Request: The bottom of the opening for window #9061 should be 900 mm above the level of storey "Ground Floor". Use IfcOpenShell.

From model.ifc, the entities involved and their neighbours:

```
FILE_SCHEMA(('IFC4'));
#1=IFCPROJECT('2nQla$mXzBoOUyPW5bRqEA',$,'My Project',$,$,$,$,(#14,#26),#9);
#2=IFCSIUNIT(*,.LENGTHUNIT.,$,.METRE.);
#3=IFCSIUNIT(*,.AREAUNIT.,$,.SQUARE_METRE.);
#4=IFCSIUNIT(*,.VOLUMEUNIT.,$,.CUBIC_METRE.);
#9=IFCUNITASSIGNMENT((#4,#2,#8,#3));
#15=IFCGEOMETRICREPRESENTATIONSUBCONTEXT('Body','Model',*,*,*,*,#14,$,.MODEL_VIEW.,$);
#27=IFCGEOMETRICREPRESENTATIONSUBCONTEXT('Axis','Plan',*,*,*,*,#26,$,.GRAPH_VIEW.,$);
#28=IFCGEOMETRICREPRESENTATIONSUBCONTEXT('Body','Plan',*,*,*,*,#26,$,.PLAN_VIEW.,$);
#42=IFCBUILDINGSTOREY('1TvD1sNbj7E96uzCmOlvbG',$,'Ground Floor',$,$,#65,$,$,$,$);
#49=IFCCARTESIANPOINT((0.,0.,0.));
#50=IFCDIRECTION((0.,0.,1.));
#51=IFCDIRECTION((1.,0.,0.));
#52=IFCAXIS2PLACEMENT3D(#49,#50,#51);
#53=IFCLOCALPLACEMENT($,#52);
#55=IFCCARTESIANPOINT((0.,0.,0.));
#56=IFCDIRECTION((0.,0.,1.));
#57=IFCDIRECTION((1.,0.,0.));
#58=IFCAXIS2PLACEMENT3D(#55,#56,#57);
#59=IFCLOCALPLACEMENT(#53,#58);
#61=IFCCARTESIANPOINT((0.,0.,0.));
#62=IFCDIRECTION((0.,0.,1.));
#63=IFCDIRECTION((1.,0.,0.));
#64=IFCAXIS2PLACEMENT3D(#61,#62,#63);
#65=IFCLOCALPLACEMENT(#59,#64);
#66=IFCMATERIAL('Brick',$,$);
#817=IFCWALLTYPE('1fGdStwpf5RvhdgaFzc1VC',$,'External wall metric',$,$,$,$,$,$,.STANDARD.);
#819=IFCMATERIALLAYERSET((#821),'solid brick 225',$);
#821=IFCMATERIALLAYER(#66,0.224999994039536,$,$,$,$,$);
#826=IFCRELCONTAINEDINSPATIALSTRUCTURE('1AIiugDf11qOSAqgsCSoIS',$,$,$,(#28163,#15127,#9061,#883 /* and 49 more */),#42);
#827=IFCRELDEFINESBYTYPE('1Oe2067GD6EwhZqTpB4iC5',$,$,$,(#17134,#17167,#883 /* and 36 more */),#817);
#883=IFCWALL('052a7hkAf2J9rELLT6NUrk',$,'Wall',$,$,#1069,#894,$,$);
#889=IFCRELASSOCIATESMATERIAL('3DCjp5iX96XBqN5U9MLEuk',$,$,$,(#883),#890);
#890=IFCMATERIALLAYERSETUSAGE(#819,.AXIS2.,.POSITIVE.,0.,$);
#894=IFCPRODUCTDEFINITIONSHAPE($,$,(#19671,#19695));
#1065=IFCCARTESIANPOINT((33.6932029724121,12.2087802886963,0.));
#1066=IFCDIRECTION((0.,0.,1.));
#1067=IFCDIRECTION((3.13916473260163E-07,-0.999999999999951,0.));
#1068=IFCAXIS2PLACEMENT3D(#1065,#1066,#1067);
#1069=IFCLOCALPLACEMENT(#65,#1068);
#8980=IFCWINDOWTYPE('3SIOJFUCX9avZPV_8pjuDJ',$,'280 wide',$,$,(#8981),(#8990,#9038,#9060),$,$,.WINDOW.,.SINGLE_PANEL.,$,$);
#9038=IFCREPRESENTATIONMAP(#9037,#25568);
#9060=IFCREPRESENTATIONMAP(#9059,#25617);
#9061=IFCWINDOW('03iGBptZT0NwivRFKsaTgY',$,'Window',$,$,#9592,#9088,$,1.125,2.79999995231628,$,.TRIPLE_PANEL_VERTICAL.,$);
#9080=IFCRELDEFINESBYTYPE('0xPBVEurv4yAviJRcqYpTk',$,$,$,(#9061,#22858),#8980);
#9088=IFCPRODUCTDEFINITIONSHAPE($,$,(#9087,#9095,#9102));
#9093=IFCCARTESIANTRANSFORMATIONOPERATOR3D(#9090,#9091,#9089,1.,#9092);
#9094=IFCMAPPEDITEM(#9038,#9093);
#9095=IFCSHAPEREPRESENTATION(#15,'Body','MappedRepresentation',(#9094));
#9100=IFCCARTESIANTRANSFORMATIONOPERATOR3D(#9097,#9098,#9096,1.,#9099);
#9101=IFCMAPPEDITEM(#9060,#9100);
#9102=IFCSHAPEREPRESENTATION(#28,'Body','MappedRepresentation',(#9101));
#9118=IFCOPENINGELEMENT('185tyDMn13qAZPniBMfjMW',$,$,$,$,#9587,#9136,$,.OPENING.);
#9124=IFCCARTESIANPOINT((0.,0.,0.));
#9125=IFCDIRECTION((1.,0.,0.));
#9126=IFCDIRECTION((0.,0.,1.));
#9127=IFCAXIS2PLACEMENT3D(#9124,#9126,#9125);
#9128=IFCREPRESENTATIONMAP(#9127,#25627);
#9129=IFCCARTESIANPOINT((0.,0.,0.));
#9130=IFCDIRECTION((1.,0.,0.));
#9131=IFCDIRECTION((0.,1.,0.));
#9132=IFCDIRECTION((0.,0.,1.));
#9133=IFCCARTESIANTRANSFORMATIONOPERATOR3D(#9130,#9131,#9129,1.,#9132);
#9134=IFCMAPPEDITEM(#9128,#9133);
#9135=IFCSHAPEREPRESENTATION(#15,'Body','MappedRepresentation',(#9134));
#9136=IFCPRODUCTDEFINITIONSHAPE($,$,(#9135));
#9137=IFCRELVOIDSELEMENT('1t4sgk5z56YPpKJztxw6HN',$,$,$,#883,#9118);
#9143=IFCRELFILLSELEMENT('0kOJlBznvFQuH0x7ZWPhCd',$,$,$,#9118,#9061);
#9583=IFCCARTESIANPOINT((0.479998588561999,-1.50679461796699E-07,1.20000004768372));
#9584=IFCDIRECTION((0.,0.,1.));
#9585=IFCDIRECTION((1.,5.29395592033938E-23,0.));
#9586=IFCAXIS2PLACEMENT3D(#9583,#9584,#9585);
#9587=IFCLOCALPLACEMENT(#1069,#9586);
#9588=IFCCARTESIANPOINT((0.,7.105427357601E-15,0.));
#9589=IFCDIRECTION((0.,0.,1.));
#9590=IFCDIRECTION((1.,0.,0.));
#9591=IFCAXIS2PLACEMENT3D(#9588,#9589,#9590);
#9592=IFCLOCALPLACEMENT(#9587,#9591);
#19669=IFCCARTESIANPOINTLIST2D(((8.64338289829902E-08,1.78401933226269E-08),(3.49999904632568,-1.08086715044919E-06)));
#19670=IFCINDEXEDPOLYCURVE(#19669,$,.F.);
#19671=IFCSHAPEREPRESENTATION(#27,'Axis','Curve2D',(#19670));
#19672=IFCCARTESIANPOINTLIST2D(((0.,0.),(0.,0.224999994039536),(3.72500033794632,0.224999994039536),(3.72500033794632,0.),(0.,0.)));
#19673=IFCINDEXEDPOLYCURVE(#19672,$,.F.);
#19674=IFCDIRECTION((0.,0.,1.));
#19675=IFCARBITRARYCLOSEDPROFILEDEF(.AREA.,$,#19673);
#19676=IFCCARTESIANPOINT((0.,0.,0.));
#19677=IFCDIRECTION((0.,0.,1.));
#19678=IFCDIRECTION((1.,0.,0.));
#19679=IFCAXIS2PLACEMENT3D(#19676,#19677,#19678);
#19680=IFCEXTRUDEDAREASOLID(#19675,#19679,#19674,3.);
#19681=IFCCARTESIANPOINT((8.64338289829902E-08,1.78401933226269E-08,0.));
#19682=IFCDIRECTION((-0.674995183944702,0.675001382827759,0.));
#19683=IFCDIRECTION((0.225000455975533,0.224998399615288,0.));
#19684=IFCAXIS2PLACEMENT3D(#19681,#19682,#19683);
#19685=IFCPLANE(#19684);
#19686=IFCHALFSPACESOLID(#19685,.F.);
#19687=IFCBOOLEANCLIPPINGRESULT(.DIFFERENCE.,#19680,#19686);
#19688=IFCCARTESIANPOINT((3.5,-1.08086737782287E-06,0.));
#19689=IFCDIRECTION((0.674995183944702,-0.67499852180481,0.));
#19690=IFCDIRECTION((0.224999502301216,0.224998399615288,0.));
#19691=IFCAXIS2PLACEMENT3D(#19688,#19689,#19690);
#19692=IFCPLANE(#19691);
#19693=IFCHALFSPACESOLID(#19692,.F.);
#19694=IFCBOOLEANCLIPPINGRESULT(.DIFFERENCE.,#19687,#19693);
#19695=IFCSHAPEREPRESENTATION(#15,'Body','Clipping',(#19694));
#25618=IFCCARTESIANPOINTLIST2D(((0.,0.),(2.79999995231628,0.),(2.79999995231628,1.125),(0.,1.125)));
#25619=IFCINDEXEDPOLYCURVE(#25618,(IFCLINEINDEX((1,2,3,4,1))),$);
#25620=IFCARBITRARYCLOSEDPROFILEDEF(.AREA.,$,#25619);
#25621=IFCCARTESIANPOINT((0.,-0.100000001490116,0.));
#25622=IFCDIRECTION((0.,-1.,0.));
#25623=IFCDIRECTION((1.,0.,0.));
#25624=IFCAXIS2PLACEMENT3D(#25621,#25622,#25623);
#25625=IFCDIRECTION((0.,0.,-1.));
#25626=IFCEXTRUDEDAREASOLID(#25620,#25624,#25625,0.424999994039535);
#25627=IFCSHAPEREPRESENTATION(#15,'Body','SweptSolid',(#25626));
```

```python
import numpy as np
import ifcopenshell
import ifcopenshell.api.geometry
import ifcopenshell.geom
import ifcopenshell.util.element
import ifcopenshell.util.placement
import ifcopenshell.util.shape
import ifcopenshell.util.unit

model = ifcopenshell.open("model.ifc")
unit_scale = ifcopenshell.util.unit.calculate_unit_scale(model)

window = model.by_guid("03iGBptZT0NwivRFKsaTgY")
opening = window.FillsVoids[0].RelatingOpeningElement
storey = ifcopenshell.util.element.get_container(window, ifc_class="IfcBuildingStorey")
level = ifcopenshell.util.placement.get_local_placement(storey.ObjectPlacement)[2, 3]

# The opening's origin need not be at the sill, so measure its lowest point.
shape = ifcopenshell.geom.create_shape(ifcopenshell.geom.settings(), opening)
bottom = ifcopenshell.util.shape.get_shape_bottom_elevation(shape, shape.geometry) / unit_scale
dz = level + 0.9 - bottom

shift = np.array([0.0, 0.0, dz])
# The window is placed relative to its opening, so it follows when the opening moves.
matrix = ifcopenshell.util.placement.get_local_placement(opening.ObjectPlacement)
matrix[:3, 3] += shift
ifcopenshell.api.geometry.edit_object_placement(
    model, product=opening, matrix=matrix, is_si=False, should_transform_children=True
)

print(f"moved by {dz * unit_scale:+.3f} m")

model.write("model_rev.ifc")
```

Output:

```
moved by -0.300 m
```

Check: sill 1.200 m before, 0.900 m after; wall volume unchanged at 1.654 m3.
